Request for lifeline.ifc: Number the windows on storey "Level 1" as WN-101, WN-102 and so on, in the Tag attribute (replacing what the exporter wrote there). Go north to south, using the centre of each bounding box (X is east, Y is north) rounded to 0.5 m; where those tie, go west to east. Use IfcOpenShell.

First a look at what the model holds.

```python
import ifcopenshell
import ifcopenshell.util.element
import ifcopenshell.util.placement

model = ifcopenshell.open("lifeline.ifc")
print(model.schema)
storey = next(s for s in model.by_type("IfcBuildingStorey") if s.Name == "Level 1")
windows = [e for e in ifcopenshell.util.element.get_decomposition(storey) if e.is_a("IfcWindow")]
for e in sorted(windows, key=lambda e: e.id()):
    origin = ifcopenshell.util.placement.get_local_placement(e.ObjectPlacement)[:3, 3]
    print(e.id(), e.Tag, e.Name, origin.round(2) + 0.0, sep=" | ")
```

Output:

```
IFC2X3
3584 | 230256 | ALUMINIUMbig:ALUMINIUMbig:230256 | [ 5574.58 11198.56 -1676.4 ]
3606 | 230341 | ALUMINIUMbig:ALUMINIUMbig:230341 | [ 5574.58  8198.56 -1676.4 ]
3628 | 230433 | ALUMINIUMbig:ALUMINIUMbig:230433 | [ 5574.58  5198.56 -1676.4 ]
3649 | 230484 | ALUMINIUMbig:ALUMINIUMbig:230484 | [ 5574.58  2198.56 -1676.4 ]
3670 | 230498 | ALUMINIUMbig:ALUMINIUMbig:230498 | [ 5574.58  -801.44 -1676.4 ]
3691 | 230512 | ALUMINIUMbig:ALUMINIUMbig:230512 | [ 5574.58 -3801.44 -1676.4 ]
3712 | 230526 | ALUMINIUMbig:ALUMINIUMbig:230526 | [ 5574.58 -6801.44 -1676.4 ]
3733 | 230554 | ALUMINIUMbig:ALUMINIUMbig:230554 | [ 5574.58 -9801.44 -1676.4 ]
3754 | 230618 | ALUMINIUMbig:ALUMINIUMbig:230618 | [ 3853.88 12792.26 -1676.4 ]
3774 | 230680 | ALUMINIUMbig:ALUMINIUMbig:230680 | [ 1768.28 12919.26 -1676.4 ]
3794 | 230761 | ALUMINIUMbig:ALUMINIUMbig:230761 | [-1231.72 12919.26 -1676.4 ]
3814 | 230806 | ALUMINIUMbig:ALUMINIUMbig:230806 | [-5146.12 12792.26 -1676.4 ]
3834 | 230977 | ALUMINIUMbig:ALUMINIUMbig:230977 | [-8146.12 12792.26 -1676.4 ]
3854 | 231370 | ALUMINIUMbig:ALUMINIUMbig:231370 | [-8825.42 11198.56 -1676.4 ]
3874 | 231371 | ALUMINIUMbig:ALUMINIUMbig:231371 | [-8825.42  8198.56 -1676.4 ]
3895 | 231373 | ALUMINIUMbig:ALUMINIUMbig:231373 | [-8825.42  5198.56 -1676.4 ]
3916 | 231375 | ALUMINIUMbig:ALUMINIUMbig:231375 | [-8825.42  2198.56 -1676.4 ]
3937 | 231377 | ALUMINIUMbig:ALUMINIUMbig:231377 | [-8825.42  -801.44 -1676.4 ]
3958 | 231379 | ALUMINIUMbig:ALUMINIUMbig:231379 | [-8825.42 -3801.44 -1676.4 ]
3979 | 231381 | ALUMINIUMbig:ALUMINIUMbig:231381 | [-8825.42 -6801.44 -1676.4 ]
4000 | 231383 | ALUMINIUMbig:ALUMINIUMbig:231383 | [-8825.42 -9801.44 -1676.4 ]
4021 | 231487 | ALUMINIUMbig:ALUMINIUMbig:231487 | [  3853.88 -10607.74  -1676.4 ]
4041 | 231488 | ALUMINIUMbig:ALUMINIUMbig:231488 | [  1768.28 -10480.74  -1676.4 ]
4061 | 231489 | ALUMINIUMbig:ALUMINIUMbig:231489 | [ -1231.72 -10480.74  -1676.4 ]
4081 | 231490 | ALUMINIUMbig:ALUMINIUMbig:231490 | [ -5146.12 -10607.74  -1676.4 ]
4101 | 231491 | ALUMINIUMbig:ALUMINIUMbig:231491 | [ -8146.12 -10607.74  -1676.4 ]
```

```python
import ifcopenshell
import ifcopenshell.geom
import ifcopenshell.util.element
import ifcopenshell.util.shape

model = ifcopenshell.open("lifeline.ifc")
settings = ifcopenshell.geom.settings()
settings.set("use-world-coords", True)


def centre(element):
    shape = ifcopenshell.geom.create_shape(settings, element)
    return ifcopenshell.util.shape.get_bbox_centroid(shape.geometry)


storey = next(s for s in model.by_type("IfcBuildingStorey") if s.Name == "Level 1")
windows = [e for e in ifcopenshell.util.element.get_decomposition(storey) if e.is_a("IfcWindow")]

# Insertion points can sit at a corner or the storey origin, so sort by the geometry (in metres).
centres = {e: centre(e) for e in windows}
windows.sort(key=lambda e: (-round(centres[e][1] / 0.5), centres[e][0]))

for i, e in enumerate(windows, start=1):
    number = f"WN-1{i:02d}"
    e.Tag = number
    print(e.id(), number)

model.write("lifeline-out.ifc")
```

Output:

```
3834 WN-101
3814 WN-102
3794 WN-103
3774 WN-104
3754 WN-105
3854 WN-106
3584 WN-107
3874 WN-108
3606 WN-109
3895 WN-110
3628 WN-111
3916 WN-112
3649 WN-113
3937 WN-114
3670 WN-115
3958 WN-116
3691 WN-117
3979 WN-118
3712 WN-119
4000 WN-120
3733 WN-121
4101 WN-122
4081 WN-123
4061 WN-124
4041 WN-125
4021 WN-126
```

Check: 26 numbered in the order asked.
